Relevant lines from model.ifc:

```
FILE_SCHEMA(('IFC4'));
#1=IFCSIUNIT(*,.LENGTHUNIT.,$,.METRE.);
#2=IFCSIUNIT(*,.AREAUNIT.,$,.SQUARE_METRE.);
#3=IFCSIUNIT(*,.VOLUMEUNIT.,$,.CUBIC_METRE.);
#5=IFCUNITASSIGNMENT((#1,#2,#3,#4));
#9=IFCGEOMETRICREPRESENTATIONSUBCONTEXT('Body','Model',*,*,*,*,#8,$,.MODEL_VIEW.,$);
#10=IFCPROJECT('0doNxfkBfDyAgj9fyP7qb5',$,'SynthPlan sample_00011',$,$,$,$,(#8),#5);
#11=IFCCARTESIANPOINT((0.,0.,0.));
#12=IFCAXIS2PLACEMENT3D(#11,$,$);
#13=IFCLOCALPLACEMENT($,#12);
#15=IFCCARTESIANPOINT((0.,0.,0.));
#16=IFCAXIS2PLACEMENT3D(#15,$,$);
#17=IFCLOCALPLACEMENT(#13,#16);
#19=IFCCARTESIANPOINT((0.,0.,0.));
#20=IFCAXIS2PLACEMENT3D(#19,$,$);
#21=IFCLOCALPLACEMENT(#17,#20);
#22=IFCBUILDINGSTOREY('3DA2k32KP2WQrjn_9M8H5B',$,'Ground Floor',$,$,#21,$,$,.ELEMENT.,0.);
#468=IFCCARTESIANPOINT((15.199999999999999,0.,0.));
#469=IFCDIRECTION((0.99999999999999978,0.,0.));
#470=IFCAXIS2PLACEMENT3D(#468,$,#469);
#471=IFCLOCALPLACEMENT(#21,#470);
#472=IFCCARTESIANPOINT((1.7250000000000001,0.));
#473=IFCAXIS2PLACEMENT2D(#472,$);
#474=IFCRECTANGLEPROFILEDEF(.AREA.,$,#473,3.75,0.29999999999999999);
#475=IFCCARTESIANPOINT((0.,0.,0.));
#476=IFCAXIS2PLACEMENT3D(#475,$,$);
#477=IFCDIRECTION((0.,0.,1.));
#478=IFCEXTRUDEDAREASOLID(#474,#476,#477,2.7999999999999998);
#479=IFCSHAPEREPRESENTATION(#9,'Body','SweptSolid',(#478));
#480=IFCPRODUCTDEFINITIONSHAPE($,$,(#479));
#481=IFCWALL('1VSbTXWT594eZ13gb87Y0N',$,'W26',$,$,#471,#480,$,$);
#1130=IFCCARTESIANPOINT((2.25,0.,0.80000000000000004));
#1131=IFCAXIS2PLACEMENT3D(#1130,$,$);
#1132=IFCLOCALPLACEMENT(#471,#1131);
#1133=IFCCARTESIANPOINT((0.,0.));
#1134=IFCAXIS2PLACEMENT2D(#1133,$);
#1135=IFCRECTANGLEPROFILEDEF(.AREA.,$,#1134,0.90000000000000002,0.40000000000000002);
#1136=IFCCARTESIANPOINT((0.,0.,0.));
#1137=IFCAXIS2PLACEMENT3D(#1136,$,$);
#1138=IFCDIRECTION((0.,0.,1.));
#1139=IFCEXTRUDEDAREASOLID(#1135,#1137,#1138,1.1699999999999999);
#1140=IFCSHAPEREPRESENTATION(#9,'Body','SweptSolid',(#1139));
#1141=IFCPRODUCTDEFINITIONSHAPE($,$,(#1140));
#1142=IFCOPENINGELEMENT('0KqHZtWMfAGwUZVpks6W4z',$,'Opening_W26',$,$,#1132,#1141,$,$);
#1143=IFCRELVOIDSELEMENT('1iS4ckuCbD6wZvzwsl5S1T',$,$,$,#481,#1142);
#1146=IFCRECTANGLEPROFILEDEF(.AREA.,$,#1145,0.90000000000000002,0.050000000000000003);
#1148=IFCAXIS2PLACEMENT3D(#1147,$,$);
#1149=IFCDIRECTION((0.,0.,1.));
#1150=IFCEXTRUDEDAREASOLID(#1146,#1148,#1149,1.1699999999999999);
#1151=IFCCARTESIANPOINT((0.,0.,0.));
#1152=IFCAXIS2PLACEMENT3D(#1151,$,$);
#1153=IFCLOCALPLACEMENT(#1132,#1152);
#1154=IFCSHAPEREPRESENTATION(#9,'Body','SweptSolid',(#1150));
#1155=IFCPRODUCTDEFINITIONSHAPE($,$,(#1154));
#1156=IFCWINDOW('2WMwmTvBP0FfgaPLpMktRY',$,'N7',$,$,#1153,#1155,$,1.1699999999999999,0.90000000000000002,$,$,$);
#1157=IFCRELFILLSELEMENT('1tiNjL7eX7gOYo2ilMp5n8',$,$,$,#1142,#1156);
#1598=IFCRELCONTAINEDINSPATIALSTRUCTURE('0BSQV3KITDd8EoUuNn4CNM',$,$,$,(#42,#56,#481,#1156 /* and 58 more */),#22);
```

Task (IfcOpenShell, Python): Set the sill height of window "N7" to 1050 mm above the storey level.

```python
import numpy as np
import ifcopenshell
import ifcopenshell.api.geometry
import ifcopenshell.geom
import ifcopenshell.util.element
import ifcopenshell.util.placement
import ifcopenshell.util.shape
import ifcopenshell.util.unit

model = ifcopenshell.open("model.ifc")
unit_scale = ifcopenshell.util.unit.calculate_unit_scale(model)

window = model.by_guid("2WMwmTvBP0FfgaPLpMktRY")
opening = window.FillsVoids[0].RelatingOpeningElement
storey = ifcopenshell.util.element.get_container(window, ifc_class="IfcBuildingStorey")
level = ifcopenshell.util.placement.get_local_placement(storey.ObjectPlacement)[2, 3]

# The opening's origin need not be at the sill, so measure its lowest point.
shape = ifcopenshell.geom.create_shape(ifcopenshell.geom.settings(), opening)
bottom = ifcopenshell.util.shape.get_shape_bottom_elevation(shape, shape.geometry) / unit_scale
dz = level + 1.05 / unit_scale - bottom

shift = np.array([0.0, 0.0, dz])
# The window is placed relative to its opening, so it follows when the opening moves.
matrix = ifcopenshell.util.placement.get_local_placement(opening.ObjectPlacement)
matrix[:3, 3] += shift
ifcopenshell.api.geometry.edit_object_placement(
    model, product=opening, matrix=matrix, is_si=False, should_transform_children=True
)

print(f"moved by {dz * unit_scale:+.3f} m")

model.write("model_updated.ifc")
```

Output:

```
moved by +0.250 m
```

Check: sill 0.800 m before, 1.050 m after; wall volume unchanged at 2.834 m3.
